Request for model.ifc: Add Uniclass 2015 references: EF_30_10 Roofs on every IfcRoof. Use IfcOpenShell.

First a look at what the model holds.

```python
import ifcopenshell

model = ifcopenshell.open("model.ifc")
print(model.schema)
print("classifications:", [c.Name for c in model.by_type("IfcClassification")])
for ifc_class in ("IfcDoor", "IfcRoof", "IfcStair", "IfcWall", "IfcWindow"):
    print(ifc_class, len(model.by_type(ifc_class)))
```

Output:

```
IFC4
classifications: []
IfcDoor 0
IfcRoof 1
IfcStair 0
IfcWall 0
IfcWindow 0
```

```python
import ifcopenshell
import ifcopenshell.api.classification

model = ifcopenshell.open("model.ifc")

system = ifcopenshell.api.classification.add_classification(model, classification="Uniclass 2015")

codes = {
    "IfcRoof": ("EF_30_10", "Roofs"),
}
for ifc_class, (code, name) in codes.items():
    products = model.by_type(ifc_class)
    ifcopenshell.api.classification.add_reference(
        model, products=products, classification=system, identification=code, name=name
    )
    print(code, len(products))

model.write("model-out.ifc")
```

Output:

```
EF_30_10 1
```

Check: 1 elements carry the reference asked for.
